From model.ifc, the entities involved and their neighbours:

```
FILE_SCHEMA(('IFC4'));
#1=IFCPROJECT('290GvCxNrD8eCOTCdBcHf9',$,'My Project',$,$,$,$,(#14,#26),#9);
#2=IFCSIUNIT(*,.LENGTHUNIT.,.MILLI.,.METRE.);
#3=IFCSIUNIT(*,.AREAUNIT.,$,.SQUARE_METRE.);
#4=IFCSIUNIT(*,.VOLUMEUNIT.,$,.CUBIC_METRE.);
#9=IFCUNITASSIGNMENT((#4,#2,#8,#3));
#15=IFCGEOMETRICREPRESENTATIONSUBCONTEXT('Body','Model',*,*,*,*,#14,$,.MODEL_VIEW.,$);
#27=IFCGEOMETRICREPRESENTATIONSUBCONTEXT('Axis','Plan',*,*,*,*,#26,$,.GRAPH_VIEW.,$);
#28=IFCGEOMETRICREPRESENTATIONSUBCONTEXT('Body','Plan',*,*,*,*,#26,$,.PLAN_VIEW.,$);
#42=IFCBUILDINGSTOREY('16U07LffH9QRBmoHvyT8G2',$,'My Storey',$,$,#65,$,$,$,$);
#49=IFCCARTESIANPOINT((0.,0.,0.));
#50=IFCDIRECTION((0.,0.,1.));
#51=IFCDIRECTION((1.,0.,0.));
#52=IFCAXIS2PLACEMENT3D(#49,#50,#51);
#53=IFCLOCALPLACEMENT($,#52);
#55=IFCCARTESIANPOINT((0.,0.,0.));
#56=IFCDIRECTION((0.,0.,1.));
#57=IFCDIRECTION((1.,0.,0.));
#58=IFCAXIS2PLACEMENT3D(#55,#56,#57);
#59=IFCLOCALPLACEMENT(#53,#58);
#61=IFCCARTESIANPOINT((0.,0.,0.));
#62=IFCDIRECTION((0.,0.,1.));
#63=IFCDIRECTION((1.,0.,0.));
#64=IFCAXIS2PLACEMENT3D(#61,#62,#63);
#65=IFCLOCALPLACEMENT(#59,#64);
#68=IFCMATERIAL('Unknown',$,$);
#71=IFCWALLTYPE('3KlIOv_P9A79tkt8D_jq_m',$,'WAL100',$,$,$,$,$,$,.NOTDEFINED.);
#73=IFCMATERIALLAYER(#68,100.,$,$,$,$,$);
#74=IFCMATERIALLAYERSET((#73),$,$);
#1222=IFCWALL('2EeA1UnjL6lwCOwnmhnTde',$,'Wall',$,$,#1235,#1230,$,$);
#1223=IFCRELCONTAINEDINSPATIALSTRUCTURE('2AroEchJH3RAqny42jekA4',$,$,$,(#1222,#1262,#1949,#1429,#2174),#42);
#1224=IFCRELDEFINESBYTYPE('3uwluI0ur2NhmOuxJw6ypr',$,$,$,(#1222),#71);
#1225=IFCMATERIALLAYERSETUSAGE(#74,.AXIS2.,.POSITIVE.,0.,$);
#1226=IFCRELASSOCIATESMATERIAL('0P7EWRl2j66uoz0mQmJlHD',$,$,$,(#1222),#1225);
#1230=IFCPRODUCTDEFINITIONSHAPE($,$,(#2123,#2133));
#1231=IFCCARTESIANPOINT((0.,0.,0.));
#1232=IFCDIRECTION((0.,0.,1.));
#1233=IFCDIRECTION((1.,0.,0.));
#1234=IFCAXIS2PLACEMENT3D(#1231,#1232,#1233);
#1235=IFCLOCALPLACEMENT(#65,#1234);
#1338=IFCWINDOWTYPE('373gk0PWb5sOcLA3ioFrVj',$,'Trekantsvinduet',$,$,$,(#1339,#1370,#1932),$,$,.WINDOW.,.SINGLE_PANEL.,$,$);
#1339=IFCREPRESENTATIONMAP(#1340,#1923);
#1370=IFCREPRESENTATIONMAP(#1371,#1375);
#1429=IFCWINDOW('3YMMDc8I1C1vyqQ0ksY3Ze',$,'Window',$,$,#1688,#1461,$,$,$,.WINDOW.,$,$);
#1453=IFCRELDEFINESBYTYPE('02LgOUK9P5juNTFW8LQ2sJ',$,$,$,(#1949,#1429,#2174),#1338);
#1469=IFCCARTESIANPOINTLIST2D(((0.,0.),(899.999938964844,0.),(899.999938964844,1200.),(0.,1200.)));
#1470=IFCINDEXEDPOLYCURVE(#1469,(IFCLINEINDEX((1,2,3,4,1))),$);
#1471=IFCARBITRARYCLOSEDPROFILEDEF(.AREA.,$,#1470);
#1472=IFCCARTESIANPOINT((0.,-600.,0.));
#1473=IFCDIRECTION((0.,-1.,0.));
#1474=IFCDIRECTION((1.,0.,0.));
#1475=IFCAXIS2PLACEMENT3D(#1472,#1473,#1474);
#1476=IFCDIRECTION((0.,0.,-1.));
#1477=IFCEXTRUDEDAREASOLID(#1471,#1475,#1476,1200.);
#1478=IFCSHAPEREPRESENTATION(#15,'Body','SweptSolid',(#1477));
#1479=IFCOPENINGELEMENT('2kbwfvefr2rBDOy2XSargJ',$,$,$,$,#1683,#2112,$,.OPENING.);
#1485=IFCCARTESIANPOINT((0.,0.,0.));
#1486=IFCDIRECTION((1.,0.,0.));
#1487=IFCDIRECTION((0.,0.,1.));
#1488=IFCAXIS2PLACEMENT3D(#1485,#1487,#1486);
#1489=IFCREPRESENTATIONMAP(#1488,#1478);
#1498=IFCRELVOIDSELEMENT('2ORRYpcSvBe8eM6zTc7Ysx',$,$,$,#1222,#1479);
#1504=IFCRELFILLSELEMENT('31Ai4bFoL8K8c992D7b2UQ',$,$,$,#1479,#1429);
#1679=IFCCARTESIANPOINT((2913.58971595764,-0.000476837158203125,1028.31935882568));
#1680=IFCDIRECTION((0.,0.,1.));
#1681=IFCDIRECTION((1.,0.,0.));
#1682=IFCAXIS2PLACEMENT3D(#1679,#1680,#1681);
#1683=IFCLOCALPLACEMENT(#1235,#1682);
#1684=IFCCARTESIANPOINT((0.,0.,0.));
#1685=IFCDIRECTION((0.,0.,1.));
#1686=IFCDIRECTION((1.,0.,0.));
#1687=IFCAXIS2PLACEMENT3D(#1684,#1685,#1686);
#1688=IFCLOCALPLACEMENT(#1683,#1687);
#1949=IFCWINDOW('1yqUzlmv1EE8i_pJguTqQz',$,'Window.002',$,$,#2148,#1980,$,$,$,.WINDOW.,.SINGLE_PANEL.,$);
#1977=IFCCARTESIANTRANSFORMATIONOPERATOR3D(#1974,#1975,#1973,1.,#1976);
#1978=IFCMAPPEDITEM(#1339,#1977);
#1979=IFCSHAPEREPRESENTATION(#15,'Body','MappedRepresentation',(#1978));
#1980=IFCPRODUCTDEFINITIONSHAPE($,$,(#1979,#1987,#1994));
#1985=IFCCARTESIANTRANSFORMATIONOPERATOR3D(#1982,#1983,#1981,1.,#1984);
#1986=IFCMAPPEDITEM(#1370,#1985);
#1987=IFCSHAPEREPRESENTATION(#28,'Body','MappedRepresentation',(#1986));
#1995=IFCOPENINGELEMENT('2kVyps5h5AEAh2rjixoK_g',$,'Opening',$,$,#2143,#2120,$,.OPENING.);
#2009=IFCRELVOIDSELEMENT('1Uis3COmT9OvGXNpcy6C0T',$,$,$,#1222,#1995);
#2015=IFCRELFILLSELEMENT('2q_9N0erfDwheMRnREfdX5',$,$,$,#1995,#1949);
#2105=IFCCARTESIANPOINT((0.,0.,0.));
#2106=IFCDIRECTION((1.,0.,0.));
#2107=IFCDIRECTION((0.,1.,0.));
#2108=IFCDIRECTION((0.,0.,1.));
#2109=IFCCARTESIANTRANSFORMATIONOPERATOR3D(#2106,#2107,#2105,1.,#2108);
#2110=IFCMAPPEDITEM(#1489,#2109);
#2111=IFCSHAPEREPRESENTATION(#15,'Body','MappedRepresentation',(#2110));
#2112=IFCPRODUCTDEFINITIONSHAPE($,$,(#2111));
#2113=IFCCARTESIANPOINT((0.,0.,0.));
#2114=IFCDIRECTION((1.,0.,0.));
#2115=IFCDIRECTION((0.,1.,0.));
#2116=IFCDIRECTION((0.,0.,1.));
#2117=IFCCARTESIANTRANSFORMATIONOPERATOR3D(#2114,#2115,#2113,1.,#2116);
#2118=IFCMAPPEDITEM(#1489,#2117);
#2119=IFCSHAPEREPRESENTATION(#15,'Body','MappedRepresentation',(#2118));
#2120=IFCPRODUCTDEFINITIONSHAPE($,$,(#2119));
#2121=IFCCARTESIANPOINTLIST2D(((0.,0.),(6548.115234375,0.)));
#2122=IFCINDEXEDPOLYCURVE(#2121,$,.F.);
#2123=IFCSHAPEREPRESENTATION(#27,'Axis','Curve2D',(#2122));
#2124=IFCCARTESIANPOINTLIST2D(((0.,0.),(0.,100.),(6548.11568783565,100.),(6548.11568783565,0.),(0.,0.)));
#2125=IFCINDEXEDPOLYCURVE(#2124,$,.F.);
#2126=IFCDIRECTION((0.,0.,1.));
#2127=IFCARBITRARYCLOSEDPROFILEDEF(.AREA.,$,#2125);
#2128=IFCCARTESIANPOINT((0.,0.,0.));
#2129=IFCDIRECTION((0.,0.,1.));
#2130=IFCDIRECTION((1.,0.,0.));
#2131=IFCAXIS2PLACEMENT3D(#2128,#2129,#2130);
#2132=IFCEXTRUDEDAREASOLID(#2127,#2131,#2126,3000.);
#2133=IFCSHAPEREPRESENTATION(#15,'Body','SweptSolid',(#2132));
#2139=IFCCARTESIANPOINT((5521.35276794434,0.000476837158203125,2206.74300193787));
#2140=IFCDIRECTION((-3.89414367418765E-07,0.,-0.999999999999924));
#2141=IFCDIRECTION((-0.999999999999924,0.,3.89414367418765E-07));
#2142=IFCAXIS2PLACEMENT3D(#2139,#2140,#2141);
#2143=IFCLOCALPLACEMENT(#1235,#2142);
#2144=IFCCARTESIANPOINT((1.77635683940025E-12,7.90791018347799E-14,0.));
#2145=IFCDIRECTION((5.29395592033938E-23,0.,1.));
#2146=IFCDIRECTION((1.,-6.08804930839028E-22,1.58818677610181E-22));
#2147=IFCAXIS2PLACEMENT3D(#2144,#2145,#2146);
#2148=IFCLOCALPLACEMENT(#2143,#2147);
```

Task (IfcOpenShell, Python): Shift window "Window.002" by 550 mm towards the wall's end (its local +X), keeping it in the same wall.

```python
import ifcopenshell
import ifcopenshell.api.geometry
import ifcopenshell.util.placement
import ifcopenshell.util.unit

model = ifcopenshell.open("model.ifc")
unit_scale = ifcopenshell.util.unit.calculate_unit_scale(model)

window = model.by_guid("1yqUzlmv1EE8i_pJguTqQz")
opening = window.FillsVoids[0].RelatingOpeningElement
wall = opening.VoidsElements[0].RelatingBuildingElement

wall_matrix = ifcopenshell.util.placement.get_local_placement(wall.ObjectPlacement)
shift = wall_matrix[:3, 0] * 0.55 / unit_scale
before = ifcopenshell.util.placement.get_local_placement(window.ObjectPlacement)[:3, 3].copy()

# The window is placed relative to its opening, so it follows when the opening moves.
matrix = ifcopenshell.util.placement.get_local_placement(opening.ObjectPlacement)
matrix[:3, 3] += shift
ifcopenshell.api.geometry.edit_object_placement(
    model, product=opening, matrix=matrix, is_si=False, should_transform_children=True
)

after = ifcopenshell.util.placement.get_local_placement(window.ObjectPlacement)[:3, 3]
print("window moved by", (after - before).round(3) + 0.0)

model.write("model_edited.ifc")
```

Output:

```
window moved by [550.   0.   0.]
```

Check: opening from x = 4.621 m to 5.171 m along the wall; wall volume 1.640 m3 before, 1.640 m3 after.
